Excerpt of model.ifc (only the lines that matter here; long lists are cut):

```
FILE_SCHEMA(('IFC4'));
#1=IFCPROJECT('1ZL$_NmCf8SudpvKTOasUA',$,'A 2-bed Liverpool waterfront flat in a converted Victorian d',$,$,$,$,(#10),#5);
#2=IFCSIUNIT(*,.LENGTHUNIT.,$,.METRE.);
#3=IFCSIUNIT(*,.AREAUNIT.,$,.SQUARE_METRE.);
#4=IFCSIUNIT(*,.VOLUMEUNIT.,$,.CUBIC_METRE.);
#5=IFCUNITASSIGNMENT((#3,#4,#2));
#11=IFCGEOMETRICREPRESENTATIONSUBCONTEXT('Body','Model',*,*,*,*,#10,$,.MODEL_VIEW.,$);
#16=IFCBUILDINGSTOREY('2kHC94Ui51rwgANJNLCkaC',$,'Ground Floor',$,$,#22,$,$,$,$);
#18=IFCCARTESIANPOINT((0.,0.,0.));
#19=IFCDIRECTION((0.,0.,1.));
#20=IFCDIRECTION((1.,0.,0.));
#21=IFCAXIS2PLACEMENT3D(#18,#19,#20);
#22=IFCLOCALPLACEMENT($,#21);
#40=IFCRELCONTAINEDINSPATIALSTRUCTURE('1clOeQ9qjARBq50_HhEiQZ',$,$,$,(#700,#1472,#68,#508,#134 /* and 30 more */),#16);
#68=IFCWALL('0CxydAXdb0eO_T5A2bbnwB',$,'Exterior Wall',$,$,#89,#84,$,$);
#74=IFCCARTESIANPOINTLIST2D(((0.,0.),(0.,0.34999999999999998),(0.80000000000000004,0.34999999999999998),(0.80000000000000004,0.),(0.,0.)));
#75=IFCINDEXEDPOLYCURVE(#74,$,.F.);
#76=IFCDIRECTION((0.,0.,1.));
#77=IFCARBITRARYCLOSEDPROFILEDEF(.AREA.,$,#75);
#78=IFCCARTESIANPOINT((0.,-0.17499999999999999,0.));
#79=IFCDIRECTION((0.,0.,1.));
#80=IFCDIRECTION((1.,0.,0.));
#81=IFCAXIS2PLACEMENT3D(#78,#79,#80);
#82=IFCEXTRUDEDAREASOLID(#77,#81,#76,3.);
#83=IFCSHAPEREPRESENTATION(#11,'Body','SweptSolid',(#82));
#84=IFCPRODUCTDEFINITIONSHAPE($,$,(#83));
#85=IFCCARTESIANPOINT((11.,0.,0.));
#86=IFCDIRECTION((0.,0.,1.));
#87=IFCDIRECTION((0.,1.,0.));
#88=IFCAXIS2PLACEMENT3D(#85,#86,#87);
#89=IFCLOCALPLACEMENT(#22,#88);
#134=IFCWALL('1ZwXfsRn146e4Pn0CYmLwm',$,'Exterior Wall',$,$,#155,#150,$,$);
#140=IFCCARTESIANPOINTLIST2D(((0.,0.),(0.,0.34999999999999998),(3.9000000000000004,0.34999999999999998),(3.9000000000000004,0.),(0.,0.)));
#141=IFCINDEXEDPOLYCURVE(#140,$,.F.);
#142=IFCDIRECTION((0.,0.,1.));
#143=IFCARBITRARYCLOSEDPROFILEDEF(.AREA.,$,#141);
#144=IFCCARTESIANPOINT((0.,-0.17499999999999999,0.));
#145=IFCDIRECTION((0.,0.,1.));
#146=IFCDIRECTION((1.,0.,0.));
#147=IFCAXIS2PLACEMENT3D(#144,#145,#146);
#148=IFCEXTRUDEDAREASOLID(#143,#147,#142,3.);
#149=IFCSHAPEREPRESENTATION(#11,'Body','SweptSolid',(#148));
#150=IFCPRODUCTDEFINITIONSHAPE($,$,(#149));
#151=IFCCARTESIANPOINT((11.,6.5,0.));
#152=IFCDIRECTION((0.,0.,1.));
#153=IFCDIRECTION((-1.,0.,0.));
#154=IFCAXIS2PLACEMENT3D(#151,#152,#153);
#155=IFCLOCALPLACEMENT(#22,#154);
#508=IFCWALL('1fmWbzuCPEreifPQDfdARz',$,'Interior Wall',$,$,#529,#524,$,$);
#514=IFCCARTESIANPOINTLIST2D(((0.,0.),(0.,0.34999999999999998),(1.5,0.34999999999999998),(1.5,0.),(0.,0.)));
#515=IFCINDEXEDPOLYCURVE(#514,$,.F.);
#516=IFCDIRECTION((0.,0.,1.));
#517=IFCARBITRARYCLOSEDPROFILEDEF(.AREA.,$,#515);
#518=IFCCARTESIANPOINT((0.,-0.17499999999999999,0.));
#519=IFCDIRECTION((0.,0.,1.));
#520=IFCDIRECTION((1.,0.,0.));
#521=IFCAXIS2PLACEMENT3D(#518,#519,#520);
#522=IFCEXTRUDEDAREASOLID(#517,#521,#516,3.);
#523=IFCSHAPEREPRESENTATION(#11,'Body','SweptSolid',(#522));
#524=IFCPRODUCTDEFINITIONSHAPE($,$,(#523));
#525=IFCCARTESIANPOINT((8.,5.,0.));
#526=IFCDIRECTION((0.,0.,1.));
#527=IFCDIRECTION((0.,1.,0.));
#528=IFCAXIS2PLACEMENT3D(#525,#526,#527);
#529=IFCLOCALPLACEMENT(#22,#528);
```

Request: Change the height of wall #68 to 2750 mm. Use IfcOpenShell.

```python
import ifcopenshell
import ifcopenshell.geom
import ifcopenshell.util.representation
import ifcopenshell.util.shape
import ifcopenshell.util.unit

model = ifcopenshell.open("model.ifc")
unit_scale = ifcopenshell.util.unit.calculate_unit_scale(model)
settings = ifcopenshell.geom.settings()


def volume(element):
    """Net volume in cubic metres, openings subtracted."""
    shape = ifcopenshell.geom.create_shape(settings, element)
    return ifcopenshell.util.shape.get_volume(shape.geometry)


wall = model.by_id(68)
before = volume(wall)

body = ifcopenshell.util.representation.get_representation(wall, "Model", "Body")
solid = body.Items[0]
old_height = solid.Depth
solid.Depth = 2.75 / unit_scale
after = volume(wall)

print(f"height {old_height:g} -> {solid.Depth:g}, volume {before:.3f} -> {after:.3f} m3")

model.write("model_rev.ifc")
```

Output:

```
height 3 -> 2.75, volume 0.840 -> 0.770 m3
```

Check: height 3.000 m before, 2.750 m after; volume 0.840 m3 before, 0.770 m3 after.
